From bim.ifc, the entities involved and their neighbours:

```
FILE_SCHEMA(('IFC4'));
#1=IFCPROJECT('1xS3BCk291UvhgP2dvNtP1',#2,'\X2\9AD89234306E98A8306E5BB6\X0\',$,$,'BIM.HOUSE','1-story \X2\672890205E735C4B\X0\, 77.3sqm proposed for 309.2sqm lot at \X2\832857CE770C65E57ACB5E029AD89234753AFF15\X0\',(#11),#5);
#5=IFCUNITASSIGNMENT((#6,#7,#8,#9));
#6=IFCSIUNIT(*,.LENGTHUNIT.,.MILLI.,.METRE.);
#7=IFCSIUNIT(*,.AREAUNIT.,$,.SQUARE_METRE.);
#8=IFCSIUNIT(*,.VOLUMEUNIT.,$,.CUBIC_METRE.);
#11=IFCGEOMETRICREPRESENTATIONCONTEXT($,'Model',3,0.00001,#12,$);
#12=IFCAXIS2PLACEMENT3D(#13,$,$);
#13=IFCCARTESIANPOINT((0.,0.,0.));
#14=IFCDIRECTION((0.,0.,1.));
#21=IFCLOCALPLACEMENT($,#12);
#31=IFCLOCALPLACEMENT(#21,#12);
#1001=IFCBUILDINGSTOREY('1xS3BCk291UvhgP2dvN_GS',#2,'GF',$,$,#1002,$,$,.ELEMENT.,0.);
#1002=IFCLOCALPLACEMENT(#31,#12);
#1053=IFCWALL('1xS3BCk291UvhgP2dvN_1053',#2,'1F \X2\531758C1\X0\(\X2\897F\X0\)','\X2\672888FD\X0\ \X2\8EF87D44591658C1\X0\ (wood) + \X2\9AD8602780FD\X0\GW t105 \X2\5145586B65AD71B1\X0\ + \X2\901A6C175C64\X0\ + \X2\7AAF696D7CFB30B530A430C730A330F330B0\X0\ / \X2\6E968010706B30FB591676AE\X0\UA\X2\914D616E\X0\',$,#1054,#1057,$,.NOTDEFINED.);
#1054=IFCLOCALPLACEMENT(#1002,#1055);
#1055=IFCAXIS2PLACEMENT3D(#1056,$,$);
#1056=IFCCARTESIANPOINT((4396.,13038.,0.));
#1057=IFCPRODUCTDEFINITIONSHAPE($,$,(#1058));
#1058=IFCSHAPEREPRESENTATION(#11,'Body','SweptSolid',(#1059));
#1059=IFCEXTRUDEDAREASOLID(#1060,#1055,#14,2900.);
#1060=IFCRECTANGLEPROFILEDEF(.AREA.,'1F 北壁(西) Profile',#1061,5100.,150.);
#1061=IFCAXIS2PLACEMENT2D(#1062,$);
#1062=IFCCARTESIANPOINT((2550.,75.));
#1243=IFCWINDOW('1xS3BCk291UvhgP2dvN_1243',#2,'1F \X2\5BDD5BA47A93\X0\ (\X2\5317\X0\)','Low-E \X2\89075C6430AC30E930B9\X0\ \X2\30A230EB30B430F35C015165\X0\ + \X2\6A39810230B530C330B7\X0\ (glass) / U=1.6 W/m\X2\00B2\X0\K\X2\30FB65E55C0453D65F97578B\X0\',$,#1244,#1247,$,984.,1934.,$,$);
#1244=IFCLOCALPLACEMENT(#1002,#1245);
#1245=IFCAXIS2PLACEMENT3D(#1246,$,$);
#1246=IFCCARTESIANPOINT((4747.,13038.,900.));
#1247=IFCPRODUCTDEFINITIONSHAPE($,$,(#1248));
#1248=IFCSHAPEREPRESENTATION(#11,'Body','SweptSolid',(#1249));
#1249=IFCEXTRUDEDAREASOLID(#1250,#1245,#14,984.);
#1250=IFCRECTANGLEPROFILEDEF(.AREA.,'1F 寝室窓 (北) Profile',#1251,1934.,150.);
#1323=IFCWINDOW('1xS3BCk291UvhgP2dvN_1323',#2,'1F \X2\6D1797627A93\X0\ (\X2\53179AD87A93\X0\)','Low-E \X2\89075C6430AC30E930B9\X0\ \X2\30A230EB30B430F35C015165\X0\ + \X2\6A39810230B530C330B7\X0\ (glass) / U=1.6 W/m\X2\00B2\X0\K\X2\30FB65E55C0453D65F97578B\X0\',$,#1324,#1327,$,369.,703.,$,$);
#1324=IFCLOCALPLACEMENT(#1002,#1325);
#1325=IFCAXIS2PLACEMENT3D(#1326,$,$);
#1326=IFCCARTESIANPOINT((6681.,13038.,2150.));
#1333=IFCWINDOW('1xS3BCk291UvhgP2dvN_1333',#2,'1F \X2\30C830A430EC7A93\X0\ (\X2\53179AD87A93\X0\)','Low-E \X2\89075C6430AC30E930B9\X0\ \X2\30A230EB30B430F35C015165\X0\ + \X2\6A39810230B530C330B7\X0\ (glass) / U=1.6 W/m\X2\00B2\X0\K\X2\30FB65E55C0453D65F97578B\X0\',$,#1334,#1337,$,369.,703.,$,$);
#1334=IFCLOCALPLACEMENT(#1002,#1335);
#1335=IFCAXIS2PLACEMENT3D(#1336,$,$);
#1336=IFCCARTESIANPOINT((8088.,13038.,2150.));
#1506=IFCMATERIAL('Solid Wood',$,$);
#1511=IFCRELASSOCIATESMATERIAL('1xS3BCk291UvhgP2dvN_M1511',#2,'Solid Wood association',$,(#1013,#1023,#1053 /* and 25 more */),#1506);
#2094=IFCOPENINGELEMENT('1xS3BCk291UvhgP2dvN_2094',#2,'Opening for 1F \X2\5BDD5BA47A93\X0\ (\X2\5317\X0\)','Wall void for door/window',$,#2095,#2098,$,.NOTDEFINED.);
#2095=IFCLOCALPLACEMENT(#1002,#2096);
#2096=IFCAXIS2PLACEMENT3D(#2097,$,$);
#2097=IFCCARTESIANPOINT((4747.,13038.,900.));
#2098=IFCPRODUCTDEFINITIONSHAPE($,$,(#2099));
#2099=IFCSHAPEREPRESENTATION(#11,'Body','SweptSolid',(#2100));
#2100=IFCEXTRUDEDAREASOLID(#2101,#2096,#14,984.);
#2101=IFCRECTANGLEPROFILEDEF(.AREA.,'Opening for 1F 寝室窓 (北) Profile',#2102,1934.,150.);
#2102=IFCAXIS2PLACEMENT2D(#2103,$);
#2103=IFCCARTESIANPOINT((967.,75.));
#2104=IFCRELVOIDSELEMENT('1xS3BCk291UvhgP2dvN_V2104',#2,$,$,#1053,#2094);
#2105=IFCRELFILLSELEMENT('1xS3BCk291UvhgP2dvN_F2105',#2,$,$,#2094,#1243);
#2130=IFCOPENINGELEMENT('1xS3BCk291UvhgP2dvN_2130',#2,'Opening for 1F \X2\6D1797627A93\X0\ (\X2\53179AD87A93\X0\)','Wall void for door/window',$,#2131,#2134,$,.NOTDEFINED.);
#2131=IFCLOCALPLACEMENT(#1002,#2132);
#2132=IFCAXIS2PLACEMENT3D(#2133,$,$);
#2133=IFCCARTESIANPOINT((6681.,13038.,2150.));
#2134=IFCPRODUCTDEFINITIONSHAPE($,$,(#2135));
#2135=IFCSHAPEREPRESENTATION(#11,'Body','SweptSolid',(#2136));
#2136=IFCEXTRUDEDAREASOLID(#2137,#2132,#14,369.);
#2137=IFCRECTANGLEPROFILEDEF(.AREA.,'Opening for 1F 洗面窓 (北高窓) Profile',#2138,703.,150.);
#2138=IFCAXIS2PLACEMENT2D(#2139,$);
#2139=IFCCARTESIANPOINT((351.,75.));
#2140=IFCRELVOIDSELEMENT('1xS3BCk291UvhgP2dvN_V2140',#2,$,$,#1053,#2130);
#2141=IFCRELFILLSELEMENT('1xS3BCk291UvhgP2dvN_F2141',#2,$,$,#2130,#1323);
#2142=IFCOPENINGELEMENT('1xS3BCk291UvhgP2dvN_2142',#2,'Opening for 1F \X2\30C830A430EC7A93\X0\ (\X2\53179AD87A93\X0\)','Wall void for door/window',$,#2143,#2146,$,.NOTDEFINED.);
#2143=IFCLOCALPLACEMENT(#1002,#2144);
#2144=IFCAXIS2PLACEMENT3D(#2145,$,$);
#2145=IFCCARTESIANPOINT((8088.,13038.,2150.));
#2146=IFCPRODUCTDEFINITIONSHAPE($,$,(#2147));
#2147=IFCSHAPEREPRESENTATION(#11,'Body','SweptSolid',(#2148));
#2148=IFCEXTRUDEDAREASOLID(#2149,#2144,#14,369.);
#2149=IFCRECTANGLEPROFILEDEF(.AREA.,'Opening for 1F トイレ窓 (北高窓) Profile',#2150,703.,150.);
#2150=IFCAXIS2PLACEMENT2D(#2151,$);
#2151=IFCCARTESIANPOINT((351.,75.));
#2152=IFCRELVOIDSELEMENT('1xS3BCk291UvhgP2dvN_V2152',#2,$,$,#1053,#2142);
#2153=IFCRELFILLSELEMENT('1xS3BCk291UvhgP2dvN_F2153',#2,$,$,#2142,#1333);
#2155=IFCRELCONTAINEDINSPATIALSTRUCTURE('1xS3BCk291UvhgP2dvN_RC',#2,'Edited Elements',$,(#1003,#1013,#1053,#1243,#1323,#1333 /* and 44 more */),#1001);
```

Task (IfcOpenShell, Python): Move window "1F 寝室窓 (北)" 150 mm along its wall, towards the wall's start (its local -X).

```python
import ifcopenshell
import ifcopenshell.api.geometry
import ifcopenshell.util.placement

model = ifcopenshell.open("bim.ifc")

window = model.by_guid("1xS3BCk291UvhgP2dvN_1243")
opening = window.FillsVoids[0].RelatingOpeningElement
wall = opening.VoidsElements[0].RelatingBuildingElement

wall_matrix = ifcopenshell.util.placement.get_local_placement(wall.ObjectPlacement)
shift = wall_matrix[:3, 0] * -150.0
before = ifcopenshell.util.placement.get_local_placement(window.ObjectPlacement)[:3, 3].copy()

# The window is not placed relative to its opening, so move both.
for product in (opening, window):
    matrix = ifcopenshell.util.placement.get_local_placement(product.ObjectPlacement)
    matrix[:3, 3] += shift
    ifcopenshell.api.geometry.edit_object_placement(model, product=product, matrix=matrix, is_si=False)

after = ifcopenshell.util.placement.get_local_placement(window.ObjectPlacement)[:3, 3]
print("window moved by", (after - before).round(3) + 0.0)

model.write("bim_updated.ifc")
```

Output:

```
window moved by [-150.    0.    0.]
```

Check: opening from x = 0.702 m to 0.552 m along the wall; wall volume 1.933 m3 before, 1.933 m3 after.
